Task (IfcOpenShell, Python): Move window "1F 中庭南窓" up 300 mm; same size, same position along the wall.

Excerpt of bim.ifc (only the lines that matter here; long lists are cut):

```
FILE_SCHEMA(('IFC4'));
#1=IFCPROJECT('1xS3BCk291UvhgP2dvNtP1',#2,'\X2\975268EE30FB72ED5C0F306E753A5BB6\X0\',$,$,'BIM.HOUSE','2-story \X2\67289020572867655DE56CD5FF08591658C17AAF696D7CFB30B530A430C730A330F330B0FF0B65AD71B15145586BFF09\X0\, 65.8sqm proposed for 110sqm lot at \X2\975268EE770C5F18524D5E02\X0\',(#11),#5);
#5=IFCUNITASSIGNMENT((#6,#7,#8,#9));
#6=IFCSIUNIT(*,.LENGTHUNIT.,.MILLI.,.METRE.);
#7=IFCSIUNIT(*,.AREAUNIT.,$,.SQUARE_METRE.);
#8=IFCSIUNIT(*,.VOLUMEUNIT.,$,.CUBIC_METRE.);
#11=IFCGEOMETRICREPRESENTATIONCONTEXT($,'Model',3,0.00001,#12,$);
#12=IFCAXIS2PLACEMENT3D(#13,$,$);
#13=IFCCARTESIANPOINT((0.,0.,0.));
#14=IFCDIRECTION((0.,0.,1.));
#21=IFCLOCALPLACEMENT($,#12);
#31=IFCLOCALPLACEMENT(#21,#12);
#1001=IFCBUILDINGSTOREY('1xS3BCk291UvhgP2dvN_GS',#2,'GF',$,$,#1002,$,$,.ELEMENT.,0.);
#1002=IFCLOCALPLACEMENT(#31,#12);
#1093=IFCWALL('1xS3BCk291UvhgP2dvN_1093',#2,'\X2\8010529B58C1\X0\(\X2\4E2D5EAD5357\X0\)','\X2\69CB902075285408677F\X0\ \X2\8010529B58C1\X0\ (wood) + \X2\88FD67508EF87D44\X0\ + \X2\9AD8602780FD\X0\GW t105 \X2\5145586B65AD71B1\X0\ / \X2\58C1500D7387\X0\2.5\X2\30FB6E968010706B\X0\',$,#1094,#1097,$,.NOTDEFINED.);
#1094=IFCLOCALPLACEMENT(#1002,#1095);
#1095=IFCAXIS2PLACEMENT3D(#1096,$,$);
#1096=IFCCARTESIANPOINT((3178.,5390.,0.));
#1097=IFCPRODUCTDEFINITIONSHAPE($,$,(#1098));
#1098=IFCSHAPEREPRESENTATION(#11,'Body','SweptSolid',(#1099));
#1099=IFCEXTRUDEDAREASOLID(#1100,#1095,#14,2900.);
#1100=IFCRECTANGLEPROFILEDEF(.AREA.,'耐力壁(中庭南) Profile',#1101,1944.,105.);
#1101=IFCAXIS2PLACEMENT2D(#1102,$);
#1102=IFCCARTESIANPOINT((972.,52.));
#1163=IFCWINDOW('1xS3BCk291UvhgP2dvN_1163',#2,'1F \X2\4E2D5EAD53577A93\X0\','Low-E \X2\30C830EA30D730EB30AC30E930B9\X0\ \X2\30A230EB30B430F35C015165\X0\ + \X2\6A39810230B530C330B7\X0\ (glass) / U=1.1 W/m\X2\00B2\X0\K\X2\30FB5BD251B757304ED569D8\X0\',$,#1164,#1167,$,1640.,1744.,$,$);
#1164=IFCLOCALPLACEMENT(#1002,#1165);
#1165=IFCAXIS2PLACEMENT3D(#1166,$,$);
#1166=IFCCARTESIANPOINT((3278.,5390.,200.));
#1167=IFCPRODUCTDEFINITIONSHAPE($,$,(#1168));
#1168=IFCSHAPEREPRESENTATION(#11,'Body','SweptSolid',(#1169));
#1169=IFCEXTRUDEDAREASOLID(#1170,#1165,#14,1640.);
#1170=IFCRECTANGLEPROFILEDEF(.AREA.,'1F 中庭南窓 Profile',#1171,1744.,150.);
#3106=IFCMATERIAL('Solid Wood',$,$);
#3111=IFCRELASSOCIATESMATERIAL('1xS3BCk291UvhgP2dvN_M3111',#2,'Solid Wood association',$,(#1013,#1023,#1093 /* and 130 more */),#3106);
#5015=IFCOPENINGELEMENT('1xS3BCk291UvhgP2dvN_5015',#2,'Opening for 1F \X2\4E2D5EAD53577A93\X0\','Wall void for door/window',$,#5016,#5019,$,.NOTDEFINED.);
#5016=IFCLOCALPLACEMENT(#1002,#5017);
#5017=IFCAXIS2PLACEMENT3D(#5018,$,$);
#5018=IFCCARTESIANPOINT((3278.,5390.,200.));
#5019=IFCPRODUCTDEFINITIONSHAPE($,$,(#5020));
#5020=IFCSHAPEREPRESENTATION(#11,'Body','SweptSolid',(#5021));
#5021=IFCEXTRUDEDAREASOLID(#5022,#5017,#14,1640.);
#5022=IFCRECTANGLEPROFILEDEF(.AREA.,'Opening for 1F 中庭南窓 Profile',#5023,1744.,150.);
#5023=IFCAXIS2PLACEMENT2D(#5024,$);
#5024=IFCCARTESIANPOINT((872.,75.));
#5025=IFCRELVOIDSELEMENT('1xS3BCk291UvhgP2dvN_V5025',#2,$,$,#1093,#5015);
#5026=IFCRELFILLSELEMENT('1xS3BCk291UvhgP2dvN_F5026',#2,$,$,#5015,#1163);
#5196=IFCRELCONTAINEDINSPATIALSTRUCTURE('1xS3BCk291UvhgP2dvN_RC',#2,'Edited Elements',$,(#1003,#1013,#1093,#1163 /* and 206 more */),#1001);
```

```python
import numpy as np
import ifcopenshell
import ifcopenshell.api.geometry
import ifcopenshell.util.placement
import ifcopenshell.util.unit

model = ifcopenshell.open("bim.ifc")
unit_scale = ifcopenshell.util.unit.calculate_unit_scale(model)

window = model.by_guid("1xS3BCk291UvhgP2dvN_1163")
opening = window.FillsVoids[0].RelatingOpeningElement
dz = 0.3 / unit_scale

shift = np.array([0.0, 0.0, dz])
# The window is not placed relative to its opening, so move both.
for product in (opening, window):
    matrix = ifcopenshell.util.placement.get_local_placement(product.ObjectPlacement)
    matrix[:3, 3] += shift
    ifcopenshell.api.geometry.edit_object_placement(model, product=product, matrix=matrix, is_si=False)

print(f"moved by {dz * unit_scale:+.3f} m")

model.write("bim_v2.ifc")
```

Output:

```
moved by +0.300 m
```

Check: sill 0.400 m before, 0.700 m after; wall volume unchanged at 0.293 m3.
